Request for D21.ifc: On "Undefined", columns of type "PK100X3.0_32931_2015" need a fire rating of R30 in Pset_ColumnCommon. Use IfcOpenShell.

First a look at what the model holds.

```python
import ifcopenshell
import ifcopenshell.util.element

model = ifcopenshell.open("D21.ifc")
print(model.schema)
storey = next(s for s in model.by_type("IfcBuildingStorey") if s.Name == "Undefined")
columns = [e for e in ifcopenshell.util.element.get_decomposition(storey) if e.is_a("IfcColumn")]
seen = {}
for e in columns:
    element_type = ifcopenshell.util.element.get_type(e)
    key = (element_type.Name if element_type != e and element_type else None, ifcopenshell.util.element.get_pset(e, "Pset_ColumnCommon", "FireRating"))
    seen[key] = seen.get(key, 0) + 1
for (name, value), count in sorted(seen.items(), key=str):
    print(count, "x", name, "|", value)
```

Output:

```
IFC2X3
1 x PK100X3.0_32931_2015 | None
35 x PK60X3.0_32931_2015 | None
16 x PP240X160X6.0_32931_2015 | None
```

```python
import ifcopenshell
import ifcopenshell.api.pset
import ifcopenshell.util.element

model = ifcopenshell.open("D21.ifc")

storey = next(s for s in model.by_type("IfcBuildingStorey") if s.Name == "Undefined")
columns = [e for e in ifcopenshell.util.element.get_decomposition(storey) if e.is_a("IfcColumn")]

count = 0
for e in columns:
    element_type = ifcopenshell.util.element.get_type(e)
    if element_type in (None, e) or element_type.Name != "PK100X3.0_32931_2015":
        continue
    # add_pset returns the element's existing set when there is one.
    pset = ifcopenshell.api.pset.add_pset(model, product=e, name="Pset_ColumnCommon")
    ifcopenshell.api.pset.edit_pset(model, pset=pset, properties={"FireRating": "R30"})
    count += 1

print(count, "columns updated")

model.write("D21_rev.ifc")
```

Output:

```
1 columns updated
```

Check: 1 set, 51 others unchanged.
